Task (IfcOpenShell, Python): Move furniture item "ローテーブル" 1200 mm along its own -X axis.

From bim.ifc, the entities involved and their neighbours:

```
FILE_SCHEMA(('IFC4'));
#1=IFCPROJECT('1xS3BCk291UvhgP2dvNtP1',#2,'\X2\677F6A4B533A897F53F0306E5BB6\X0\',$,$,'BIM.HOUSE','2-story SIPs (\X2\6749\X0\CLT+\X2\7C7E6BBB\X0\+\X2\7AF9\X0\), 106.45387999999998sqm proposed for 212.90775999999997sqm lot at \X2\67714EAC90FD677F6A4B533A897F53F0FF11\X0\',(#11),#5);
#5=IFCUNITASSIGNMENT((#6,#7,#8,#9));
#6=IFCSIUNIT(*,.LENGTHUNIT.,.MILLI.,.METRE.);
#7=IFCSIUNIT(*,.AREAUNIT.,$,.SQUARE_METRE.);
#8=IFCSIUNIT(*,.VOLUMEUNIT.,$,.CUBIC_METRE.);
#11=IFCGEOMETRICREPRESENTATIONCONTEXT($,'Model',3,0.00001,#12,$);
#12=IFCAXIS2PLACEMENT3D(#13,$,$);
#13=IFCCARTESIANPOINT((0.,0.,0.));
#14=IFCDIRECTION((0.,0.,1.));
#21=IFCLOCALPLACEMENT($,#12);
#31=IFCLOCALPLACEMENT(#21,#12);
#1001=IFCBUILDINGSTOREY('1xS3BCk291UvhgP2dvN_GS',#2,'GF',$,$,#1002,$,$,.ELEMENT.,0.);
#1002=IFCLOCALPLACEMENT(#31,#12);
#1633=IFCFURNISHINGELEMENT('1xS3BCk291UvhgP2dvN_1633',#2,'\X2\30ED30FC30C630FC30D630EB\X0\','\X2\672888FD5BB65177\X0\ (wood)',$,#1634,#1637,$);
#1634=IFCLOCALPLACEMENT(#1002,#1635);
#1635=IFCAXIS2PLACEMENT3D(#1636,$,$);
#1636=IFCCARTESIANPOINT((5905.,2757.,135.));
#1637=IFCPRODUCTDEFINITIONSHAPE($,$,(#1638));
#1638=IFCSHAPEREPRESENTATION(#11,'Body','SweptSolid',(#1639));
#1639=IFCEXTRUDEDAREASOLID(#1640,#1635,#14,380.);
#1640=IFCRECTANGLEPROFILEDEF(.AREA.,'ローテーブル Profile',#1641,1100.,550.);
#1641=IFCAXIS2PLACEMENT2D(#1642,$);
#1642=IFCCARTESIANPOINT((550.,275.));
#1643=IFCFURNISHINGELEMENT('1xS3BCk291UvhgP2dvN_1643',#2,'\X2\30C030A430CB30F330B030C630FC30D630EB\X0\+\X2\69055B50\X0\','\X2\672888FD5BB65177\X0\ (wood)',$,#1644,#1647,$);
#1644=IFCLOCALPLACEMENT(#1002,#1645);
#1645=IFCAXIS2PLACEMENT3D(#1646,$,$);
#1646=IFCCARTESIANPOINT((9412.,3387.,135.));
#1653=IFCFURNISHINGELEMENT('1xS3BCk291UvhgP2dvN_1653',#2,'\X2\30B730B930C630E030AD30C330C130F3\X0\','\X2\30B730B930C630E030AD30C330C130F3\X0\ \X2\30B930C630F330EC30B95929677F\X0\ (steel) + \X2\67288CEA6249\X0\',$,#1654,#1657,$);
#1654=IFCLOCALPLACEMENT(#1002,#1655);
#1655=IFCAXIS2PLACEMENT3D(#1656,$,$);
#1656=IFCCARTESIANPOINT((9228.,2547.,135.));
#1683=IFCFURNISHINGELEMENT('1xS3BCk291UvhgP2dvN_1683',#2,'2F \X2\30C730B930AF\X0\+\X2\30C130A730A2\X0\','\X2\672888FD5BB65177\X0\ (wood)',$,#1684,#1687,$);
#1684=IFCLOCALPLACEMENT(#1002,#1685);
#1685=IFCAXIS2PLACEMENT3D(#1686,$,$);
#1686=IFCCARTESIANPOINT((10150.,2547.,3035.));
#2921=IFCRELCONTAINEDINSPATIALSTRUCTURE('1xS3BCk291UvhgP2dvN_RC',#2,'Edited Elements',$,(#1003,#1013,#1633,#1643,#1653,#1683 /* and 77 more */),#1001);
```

```python
import ifcopenshell
import ifcopenshell.api.geometry
import ifcopenshell.util.placement
import ifcopenshell.util.unit

model = ifcopenshell.open("bim.ifc")
unit_scale = ifcopenshell.util.unit.calculate_unit_scale(model)

item = model.by_guid("1xS3BCk291UvhgP2dvN_1633")
matrix = ifcopenshell.util.placement.get_local_placement(item.ObjectPlacement)
matrix[:3, 3] -= matrix[:3, 0] * 1.2 / unit_scale
ifcopenshell.api.geometry.edit_object_placement(model, product=item, matrix=matrix, is_si=False)

print(ifcopenshell.util.placement.get_local_placement(item.ObjectPlacement).round(3) + 0.0)

model.write("bim_updated.ifc")
```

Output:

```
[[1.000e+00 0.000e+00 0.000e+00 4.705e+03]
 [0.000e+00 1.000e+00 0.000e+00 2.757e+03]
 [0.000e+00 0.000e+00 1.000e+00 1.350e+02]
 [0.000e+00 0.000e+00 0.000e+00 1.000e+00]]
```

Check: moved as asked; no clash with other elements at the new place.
